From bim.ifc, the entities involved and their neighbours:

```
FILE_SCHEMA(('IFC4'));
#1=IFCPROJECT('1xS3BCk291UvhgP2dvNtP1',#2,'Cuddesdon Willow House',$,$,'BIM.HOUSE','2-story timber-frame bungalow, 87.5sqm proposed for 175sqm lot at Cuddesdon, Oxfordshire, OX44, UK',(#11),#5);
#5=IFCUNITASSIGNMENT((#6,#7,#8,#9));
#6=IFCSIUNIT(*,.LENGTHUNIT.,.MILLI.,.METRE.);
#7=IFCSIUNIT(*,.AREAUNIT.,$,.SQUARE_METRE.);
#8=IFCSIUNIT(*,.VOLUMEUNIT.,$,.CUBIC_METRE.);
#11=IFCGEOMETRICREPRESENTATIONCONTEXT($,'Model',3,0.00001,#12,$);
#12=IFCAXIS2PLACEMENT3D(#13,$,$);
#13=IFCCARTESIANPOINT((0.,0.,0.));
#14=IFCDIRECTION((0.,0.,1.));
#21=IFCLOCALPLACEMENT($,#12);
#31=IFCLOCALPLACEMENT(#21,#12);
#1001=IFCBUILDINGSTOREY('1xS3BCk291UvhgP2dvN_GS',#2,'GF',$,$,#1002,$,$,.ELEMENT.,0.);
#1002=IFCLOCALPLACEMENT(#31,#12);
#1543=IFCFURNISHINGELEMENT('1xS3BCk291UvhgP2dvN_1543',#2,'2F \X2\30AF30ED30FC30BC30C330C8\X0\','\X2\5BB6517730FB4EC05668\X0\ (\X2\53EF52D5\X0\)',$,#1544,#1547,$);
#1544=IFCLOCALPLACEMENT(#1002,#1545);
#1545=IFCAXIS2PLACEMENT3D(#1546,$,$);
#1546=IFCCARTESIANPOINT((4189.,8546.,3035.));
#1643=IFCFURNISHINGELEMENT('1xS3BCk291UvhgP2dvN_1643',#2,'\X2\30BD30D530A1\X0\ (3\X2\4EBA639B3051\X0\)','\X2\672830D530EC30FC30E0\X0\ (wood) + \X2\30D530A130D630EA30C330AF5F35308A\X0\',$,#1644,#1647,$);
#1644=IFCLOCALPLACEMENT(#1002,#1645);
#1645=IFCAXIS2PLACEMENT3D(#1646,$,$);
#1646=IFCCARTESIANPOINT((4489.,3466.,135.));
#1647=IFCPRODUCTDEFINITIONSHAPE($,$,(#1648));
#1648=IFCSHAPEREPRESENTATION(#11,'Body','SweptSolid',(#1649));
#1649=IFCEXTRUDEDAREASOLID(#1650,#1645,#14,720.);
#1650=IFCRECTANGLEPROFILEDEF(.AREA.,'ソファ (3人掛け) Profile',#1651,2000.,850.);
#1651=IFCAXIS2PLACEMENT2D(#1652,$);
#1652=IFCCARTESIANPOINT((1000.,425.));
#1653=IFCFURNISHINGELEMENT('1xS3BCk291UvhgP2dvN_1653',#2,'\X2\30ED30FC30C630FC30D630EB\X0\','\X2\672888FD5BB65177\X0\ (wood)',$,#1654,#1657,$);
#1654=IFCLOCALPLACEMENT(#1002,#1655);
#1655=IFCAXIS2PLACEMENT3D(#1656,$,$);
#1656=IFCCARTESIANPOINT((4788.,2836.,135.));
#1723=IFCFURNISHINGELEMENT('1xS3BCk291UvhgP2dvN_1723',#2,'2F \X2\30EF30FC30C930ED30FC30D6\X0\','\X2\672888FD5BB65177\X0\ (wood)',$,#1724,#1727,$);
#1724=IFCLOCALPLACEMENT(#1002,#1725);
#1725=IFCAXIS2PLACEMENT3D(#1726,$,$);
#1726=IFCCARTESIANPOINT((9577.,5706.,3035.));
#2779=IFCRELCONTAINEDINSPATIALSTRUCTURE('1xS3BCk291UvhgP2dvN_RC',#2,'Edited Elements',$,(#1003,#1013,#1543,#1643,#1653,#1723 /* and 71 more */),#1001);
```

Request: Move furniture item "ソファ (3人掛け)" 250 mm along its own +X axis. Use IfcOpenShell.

```python
import ifcopenshell
import ifcopenshell.api.geometry
import ifcopenshell.util.placement

model = ifcopenshell.open("bim.ifc")

item = model.by_guid("1xS3BCk291UvhgP2dvN_1643")
matrix = ifcopenshell.util.placement.get_local_placement(item.ObjectPlacement)
matrix[:3, 3] += matrix[:3, 0] * 250.0
ifcopenshell.api.geometry.edit_object_placement(model, product=item, matrix=matrix, is_si=False)

print(ifcopenshell.util.placement.get_local_placement(item.ObjectPlacement).round(3) + 0.0)

model.write("bim_updated.ifc")
```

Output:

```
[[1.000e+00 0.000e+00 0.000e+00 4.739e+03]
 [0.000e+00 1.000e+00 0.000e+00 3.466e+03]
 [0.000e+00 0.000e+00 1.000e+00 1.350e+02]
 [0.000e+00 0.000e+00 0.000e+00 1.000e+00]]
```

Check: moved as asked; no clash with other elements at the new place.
